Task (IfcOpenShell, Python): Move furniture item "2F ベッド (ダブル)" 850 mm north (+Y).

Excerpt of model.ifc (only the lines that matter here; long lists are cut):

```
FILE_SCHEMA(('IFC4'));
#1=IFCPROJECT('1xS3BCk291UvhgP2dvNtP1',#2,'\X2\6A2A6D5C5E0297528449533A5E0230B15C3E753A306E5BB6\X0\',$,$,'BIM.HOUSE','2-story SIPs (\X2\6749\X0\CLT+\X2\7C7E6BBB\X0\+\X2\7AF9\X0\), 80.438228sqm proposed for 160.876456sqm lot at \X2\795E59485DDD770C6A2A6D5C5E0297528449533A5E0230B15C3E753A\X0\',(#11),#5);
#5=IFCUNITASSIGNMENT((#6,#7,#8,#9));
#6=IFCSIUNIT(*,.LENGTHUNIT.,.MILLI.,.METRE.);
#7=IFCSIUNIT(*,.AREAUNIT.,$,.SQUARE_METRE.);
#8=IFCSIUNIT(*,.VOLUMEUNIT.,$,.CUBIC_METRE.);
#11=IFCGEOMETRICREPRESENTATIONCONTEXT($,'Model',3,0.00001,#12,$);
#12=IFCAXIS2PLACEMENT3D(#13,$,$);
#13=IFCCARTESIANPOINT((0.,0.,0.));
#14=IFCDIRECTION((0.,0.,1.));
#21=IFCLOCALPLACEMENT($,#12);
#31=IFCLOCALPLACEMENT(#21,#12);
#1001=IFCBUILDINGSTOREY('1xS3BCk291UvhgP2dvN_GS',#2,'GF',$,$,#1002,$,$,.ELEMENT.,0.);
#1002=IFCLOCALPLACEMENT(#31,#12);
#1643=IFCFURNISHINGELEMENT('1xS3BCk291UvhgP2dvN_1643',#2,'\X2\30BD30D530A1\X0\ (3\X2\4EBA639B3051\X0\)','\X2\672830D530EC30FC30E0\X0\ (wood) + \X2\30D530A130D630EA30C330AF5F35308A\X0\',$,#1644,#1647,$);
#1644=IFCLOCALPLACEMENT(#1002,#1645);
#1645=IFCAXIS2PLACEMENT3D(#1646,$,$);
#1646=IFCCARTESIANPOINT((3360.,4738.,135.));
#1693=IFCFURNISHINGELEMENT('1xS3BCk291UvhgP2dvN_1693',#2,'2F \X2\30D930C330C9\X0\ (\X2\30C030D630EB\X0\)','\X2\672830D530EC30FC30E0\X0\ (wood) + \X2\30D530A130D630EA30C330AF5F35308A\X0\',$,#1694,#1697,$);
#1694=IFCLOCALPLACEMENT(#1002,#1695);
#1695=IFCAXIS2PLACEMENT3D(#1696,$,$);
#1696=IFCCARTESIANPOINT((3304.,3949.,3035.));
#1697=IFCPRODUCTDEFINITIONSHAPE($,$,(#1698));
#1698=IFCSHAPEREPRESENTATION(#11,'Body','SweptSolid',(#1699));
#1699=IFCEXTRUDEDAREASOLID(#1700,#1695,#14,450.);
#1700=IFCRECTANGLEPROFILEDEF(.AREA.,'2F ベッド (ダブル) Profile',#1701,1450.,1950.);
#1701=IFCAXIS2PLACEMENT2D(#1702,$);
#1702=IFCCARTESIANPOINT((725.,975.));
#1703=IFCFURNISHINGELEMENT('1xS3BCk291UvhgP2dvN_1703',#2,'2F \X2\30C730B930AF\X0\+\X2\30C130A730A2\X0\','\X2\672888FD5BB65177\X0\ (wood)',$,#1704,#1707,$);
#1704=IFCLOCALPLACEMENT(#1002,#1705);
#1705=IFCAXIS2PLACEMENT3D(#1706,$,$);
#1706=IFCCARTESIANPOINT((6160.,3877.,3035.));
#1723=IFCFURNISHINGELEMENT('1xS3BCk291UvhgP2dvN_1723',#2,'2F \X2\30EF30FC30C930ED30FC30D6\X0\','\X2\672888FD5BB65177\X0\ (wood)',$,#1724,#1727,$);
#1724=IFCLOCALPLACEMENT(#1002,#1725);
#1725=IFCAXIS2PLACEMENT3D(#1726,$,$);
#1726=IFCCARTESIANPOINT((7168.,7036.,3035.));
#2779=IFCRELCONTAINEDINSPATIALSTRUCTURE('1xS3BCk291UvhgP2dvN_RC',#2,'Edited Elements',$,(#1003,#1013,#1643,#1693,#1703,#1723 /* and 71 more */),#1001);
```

```python
import ifcopenshell
import ifcopenshell.api.geometry
import ifcopenshell.util.placement
import ifcopenshell.util.unit

model = ifcopenshell.open("model.ifc")
unit_scale = ifcopenshell.util.unit.calculate_unit_scale(model)

item = model.by_guid("1xS3BCk291UvhgP2dvN_1693")
matrix = ifcopenshell.util.placement.get_local_placement(item.ObjectPlacement)
matrix[1, 3] += 0.85 / unit_scale
ifcopenshell.api.geometry.edit_object_placement(model, product=item, matrix=matrix, is_si=False)

print(ifcopenshell.util.placement.get_local_placement(item.ObjectPlacement).round(3) + 0.0)

model.write("model_edited.ifc")
```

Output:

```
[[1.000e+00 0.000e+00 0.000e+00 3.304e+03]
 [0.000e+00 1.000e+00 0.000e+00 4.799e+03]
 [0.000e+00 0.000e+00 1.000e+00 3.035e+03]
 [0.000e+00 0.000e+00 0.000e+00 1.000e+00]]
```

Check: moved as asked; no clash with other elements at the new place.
